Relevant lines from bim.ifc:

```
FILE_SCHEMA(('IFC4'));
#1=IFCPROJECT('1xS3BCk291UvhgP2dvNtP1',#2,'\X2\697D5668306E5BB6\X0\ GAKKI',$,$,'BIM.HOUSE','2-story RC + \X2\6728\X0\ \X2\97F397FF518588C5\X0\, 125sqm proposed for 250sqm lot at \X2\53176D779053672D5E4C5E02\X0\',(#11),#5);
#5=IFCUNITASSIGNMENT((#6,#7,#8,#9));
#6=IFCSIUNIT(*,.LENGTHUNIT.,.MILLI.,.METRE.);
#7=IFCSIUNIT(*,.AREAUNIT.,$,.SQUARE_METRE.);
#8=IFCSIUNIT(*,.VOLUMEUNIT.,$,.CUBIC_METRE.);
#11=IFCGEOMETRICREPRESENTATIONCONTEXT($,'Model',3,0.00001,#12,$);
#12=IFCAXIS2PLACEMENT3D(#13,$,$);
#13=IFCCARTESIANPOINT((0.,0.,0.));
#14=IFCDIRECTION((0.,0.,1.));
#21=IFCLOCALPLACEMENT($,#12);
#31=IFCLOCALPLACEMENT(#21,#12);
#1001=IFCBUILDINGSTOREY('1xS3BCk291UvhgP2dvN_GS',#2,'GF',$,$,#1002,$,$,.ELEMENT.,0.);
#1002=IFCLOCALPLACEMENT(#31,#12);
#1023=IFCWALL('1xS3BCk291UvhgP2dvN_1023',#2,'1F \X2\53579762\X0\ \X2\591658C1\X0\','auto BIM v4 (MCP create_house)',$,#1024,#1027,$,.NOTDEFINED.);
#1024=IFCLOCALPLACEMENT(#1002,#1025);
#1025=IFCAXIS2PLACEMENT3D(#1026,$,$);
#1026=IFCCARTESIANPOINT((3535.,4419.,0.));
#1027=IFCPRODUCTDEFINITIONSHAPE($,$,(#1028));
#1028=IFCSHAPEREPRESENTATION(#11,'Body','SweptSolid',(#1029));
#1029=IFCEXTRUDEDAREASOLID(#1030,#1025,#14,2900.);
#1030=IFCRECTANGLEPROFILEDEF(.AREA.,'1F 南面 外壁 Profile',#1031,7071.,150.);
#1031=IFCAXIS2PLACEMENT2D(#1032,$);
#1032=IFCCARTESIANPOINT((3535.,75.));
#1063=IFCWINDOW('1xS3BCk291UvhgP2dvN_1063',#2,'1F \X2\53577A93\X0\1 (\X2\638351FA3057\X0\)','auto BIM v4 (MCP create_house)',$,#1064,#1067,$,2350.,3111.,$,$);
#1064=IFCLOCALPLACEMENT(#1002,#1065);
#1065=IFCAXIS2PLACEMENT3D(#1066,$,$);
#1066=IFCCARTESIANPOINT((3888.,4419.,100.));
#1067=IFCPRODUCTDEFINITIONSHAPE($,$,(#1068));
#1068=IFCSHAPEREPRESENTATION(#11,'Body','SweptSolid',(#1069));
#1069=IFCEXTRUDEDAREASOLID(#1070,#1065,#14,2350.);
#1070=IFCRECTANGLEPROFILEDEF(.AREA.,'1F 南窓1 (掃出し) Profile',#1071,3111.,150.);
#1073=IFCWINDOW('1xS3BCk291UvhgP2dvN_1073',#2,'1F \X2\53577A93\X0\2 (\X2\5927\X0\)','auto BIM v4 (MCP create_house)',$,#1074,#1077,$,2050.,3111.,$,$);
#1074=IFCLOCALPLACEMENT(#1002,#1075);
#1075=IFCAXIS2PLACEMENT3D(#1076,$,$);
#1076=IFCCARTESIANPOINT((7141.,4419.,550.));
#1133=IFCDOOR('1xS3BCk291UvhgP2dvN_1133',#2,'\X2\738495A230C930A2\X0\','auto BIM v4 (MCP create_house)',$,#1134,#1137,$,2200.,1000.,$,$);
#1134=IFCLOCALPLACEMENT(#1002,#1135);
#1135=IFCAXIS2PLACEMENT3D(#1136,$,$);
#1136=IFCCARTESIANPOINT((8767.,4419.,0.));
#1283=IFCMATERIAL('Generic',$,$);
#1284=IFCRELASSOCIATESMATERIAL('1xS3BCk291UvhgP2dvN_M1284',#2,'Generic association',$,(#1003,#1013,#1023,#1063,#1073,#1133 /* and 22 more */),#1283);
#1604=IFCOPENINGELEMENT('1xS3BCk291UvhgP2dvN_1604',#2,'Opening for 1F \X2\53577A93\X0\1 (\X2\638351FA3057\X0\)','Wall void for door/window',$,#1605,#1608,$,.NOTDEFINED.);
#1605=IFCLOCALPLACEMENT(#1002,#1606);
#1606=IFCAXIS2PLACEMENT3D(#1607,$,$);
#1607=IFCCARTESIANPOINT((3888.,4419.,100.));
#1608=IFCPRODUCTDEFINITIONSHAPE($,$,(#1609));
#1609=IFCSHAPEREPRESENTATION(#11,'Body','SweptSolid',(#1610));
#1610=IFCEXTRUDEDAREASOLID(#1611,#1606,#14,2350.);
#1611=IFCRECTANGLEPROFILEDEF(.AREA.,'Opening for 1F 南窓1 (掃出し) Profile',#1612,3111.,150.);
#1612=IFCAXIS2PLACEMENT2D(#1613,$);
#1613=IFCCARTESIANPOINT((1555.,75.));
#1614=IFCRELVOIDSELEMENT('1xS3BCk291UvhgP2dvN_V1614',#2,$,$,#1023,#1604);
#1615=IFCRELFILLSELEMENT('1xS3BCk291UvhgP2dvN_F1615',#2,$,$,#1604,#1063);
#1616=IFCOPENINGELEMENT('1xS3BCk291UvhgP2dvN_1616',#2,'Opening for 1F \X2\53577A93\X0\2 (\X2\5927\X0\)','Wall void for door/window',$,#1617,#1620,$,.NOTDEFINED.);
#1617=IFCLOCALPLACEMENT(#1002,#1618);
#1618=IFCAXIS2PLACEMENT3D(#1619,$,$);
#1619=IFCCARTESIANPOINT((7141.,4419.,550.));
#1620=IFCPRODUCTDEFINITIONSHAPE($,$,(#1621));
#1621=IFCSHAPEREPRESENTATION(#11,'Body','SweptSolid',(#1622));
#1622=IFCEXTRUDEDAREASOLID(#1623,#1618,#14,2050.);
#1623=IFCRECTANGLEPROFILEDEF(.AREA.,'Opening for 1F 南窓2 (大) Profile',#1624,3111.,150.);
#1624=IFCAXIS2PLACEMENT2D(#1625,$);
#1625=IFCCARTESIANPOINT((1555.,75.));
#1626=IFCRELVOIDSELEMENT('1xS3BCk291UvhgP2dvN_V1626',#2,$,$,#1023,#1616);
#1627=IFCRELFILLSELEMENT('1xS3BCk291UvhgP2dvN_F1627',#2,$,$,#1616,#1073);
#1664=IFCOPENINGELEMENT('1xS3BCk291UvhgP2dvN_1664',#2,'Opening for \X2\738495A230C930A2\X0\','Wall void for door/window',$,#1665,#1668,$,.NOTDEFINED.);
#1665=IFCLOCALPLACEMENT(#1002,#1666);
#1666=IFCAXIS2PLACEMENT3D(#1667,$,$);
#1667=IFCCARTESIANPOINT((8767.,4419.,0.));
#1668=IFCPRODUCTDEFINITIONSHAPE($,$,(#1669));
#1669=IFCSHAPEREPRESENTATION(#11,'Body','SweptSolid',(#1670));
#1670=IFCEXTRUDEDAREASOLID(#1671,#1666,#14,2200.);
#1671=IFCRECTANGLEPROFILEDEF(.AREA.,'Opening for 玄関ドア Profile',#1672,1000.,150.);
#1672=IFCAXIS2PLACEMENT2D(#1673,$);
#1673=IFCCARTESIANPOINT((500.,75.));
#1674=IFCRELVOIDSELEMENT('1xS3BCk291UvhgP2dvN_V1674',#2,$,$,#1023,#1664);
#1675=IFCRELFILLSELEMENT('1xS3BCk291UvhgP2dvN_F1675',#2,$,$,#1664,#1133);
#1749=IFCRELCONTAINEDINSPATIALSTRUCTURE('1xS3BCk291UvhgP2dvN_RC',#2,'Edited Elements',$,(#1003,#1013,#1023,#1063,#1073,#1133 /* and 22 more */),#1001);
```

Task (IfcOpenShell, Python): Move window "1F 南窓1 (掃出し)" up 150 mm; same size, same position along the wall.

```python
import numpy as np
import ifcopenshell
import ifcopenshell.api.geometry
import ifcopenshell.util.placement
import ifcopenshell.util.unit

model = ifcopenshell.open("bim.ifc")
unit_scale = ifcopenshell.util.unit.calculate_unit_scale(model)

window = model.by_guid("1xS3BCk291UvhgP2dvN_1063")
opening = window.FillsVoids[0].RelatingOpeningElement
dz = 0.15 / unit_scale

shift = np.array([0.0, 0.0, dz])
# The window is not placed relative to its opening, so move both.
for product in (opening, window):
    matrix = ifcopenshell.util.placement.get_local_placement(product.ObjectPlacement)
    matrix[:3, 3] += shift
    ifcopenshell.api.geometry.edit_object_placement(model, product=product, matrix=matrix, is_si=False)

print(f"moved by {dz * unit_scale:+.3f} m")

model.write("bim_updated.ifc")
```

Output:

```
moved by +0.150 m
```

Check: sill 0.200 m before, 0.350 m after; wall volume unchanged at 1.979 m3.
